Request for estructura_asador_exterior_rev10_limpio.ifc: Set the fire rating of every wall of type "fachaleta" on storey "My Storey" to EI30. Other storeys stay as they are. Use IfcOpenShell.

First a look at what the model holds.

```python
import ifcopenshell
import ifcopenshell.util.element

model = ifcopenshell.open("estructura_asador_exterior_rev10_limpio.ifc")
print(model.schema)
storey = next(s for s in model.by_type("IfcBuildingStorey") if s.Name == "My Storey")
walls = [e for e in ifcopenshell.util.element.get_decomposition(storey) if e.is_a("IfcWall")]
seen = {}
for e in walls:
    element_type = ifcopenshell.util.element.get_type(e)
    key = (element_type.Name if element_type != e and element_type else None, ifcopenshell.util.element.get_pset(e, "Pset_WallCommon", "FireRating"))
    seen[key] = seen.get(key, 0) + 1
for (name, value), count in sorted(seen.items(), key=str):
    print(count, "x", name, "|", value)
```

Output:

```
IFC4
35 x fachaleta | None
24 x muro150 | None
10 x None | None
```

```python
import ifcopenshell
import ifcopenshell.api.pset
import ifcopenshell.util.element

model = ifcopenshell.open("estructura_asador_exterior_rev10_limpio.ifc")

storey = next(s for s in model.by_type("IfcBuildingStorey") if s.Name == "My Storey")
walls = [e for e in ifcopenshell.util.element.get_decomposition(storey) if e.is_a("IfcWall")]

count = 0
for e in walls:
    element_type = ifcopenshell.util.element.get_type(e)
    if element_type in (None, e) or element_type.Name != "fachaleta":
        continue
    # add_pset returns the element's existing set when there is one.
    pset = ifcopenshell.api.pset.add_pset(model, product=e, name="Pset_WallCommon")
    ifcopenshell.api.pset.edit_pset(model, pset=pset, properties={"FireRating": "EI30"})
    count += 1

print(count, "walls updated")

model.write("estructura_asador_exterior_rev10_limpio-out.ifc")
```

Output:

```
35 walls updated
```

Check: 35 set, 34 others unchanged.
